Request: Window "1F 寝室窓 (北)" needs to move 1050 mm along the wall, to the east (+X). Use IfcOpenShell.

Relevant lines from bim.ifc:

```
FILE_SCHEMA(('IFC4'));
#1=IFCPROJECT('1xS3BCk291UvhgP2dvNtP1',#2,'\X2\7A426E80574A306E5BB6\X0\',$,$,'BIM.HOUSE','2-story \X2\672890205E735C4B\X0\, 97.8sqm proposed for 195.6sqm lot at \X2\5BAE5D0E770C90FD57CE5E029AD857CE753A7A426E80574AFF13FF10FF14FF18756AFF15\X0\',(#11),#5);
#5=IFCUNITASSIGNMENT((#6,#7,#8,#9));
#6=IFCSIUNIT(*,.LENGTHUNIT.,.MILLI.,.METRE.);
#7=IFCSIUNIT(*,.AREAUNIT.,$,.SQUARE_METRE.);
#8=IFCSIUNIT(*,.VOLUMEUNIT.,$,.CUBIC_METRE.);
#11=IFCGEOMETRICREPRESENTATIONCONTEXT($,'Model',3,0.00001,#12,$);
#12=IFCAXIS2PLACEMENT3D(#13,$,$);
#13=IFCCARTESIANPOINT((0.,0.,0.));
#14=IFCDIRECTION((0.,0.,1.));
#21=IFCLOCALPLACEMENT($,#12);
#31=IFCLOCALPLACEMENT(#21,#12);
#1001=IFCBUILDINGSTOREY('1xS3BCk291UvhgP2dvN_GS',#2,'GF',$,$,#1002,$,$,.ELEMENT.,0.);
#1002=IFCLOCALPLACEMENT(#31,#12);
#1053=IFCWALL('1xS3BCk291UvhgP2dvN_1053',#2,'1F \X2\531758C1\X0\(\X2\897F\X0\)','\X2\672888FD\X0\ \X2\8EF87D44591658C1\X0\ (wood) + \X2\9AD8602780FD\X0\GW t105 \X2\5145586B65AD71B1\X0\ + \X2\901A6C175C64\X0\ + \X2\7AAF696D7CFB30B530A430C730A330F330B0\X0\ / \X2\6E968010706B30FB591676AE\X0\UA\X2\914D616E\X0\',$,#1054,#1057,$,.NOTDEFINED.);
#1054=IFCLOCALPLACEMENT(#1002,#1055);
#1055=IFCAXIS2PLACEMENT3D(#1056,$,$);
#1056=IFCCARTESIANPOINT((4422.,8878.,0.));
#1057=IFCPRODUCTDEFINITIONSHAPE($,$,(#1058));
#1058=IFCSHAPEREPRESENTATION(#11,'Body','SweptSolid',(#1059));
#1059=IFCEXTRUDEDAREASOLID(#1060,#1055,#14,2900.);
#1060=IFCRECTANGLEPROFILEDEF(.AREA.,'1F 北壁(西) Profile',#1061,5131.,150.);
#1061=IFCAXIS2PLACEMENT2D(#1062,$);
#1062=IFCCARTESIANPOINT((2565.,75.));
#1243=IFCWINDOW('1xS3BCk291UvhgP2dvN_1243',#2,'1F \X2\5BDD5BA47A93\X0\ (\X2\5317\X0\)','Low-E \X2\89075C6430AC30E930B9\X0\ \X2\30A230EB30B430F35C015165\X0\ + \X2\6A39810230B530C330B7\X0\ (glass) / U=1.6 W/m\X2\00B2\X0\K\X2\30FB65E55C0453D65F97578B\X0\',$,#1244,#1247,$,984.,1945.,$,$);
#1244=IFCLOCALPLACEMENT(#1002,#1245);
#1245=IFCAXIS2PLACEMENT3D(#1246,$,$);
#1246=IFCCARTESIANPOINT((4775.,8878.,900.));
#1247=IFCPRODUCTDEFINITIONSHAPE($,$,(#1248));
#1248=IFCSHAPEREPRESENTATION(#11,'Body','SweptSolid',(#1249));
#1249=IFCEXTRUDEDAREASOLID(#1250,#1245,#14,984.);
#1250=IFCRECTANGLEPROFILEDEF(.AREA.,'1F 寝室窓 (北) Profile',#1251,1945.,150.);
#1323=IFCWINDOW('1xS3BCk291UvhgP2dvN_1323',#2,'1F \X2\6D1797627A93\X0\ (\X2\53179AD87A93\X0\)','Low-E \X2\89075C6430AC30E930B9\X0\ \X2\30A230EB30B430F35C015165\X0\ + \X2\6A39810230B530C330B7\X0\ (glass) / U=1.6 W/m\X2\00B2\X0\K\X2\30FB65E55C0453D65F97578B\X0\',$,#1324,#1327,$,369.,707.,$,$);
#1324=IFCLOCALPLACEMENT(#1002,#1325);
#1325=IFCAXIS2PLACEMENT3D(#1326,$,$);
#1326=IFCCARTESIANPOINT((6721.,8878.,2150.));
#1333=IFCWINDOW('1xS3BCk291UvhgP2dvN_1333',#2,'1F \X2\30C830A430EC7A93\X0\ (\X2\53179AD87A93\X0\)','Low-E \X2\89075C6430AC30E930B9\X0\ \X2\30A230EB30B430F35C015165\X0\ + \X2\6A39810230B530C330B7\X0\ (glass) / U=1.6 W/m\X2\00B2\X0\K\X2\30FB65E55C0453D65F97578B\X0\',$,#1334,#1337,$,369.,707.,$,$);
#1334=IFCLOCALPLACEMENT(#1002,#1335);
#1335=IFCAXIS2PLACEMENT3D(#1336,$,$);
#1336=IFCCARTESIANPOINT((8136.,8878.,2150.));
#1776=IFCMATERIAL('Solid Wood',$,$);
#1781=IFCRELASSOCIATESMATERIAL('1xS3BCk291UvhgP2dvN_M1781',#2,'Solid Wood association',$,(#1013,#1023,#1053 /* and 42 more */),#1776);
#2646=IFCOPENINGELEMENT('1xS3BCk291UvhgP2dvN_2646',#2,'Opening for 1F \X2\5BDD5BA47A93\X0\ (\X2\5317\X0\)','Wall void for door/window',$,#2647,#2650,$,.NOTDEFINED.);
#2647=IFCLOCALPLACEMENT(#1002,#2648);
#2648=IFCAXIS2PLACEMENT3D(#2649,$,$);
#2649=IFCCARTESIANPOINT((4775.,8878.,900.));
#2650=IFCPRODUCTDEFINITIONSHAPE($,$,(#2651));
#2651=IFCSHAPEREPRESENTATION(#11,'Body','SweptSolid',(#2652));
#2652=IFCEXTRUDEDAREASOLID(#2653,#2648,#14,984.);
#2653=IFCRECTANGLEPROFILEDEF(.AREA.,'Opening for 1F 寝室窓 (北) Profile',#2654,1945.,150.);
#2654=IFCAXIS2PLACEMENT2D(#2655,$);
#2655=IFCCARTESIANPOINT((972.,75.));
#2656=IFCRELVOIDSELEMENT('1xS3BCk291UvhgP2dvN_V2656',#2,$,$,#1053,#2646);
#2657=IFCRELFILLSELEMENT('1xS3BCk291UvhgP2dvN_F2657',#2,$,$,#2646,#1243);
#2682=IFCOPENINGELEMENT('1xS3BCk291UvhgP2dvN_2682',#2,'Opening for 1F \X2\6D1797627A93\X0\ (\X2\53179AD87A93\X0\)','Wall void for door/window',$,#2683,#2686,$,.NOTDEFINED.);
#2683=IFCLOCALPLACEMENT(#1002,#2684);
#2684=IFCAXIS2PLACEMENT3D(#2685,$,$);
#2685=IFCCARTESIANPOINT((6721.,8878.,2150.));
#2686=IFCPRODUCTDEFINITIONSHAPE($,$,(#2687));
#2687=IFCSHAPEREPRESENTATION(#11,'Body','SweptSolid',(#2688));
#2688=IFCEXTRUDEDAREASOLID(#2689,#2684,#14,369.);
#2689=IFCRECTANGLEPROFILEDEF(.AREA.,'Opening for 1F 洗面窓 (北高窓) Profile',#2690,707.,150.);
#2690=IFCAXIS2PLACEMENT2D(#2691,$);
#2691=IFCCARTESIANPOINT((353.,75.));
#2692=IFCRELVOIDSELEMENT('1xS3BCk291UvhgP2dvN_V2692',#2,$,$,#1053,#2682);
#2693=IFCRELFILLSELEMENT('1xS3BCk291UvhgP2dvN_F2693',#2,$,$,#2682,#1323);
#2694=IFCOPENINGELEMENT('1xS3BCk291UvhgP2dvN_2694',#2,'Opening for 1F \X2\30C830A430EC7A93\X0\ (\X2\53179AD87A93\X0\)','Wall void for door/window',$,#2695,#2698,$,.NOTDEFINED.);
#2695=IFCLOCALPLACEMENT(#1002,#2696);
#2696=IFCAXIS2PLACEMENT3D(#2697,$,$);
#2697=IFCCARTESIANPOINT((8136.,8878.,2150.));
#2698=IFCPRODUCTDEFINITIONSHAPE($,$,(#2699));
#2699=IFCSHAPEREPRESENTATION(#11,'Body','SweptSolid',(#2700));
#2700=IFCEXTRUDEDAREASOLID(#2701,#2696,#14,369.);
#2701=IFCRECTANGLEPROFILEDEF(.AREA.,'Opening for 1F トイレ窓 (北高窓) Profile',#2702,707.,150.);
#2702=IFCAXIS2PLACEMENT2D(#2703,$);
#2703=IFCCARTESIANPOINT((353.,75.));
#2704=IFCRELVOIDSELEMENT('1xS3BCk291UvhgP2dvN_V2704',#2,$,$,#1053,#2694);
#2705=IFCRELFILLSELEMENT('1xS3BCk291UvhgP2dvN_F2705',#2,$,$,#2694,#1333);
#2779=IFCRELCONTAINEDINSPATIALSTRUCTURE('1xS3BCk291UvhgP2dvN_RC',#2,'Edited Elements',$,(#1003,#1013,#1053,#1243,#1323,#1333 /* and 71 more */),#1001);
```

```python
import ifcopenshell
import ifcopenshell.api.geometry
import ifcopenshell.util.placement
import ifcopenshell.util.unit

model = ifcopenshell.open("bim.ifc")
unit_scale = ifcopenshell.util.unit.calculate_unit_scale(model)

window = model.by_id(1243)
opening = window.FillsVoids[0].RelatingOpeningElement
wall = opening.VoidsElements[0].RelatingBuildingElement

wall_matrix = ifcopenshell.util.placement.get_local_placement(wall.ObjectPlacement)
shift = wall_matrix[:3, 0] * 1.05 / unit_scale
before = ifcopenshell.util.placement.get_local_placement(window.ObjectPlacement)[:3, 3].copy()

# The window is not placed relative to its opening, so move both.
for product in (opening, window):
    matrix = ifcopenshell.util.placement.get_local_placement(product.ObjectPlacement)
    matrix[:3, 3] += shift
    ifcopenshell.api.geometry.edit_object_placement(model, product=product, matrix=matrix, is_si=False)

after = ifcopenshell.util.placement.get_local_placement(window.ObjectPlacement)[:3, 3]
print("window moved by", (after - before).round(3) + 0.0)

model.write("bim-out.ifc")
```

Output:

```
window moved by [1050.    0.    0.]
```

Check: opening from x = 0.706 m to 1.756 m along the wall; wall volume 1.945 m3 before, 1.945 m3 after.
